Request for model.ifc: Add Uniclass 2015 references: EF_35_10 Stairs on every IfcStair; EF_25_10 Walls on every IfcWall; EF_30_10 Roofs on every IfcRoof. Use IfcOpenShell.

First a look at what the model holds.

```python
import ifcopenshell

model = ifcopenshell.open("model.ifc")
print(model.schema)
print("classifications:", [c.Name for c in model.by_type("IfcClassification")])
for ifc_class in ("IfcDoor", "IfcRoof", "IfcStair", "IfcWall", "IfcWindow"):
    print(ifc_class, len(model.by_type(ifc_class)))
```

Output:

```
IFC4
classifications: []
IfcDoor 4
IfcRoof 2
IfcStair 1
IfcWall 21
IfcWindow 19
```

```python
import ifcopenshell
import ifcopenshell.api.classification

model = ifcopenshell.open("model.ifc")

system = ifcopenshell.api.classification.add_classification(model, classification="Uniclass 2015")

codes = {
    "IfcStair": ("EF_35_10", "Stairs"),
    "IfcWall": ("EF_25_10", "Walls"),
    "IfcRoof": ("EF_30_10", "Roofs"),
}
for ifc_class, (code, name) in codes.items():
    products = model.by_type(ifc_class)
    ifcopenshell.api.classification.add_reference(
        model, products=products, classification=system, identification=code, name=name
    )
    print(code, len(products))

model.write("model-out.ifc")
```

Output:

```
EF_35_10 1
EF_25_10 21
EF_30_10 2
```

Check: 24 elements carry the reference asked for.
